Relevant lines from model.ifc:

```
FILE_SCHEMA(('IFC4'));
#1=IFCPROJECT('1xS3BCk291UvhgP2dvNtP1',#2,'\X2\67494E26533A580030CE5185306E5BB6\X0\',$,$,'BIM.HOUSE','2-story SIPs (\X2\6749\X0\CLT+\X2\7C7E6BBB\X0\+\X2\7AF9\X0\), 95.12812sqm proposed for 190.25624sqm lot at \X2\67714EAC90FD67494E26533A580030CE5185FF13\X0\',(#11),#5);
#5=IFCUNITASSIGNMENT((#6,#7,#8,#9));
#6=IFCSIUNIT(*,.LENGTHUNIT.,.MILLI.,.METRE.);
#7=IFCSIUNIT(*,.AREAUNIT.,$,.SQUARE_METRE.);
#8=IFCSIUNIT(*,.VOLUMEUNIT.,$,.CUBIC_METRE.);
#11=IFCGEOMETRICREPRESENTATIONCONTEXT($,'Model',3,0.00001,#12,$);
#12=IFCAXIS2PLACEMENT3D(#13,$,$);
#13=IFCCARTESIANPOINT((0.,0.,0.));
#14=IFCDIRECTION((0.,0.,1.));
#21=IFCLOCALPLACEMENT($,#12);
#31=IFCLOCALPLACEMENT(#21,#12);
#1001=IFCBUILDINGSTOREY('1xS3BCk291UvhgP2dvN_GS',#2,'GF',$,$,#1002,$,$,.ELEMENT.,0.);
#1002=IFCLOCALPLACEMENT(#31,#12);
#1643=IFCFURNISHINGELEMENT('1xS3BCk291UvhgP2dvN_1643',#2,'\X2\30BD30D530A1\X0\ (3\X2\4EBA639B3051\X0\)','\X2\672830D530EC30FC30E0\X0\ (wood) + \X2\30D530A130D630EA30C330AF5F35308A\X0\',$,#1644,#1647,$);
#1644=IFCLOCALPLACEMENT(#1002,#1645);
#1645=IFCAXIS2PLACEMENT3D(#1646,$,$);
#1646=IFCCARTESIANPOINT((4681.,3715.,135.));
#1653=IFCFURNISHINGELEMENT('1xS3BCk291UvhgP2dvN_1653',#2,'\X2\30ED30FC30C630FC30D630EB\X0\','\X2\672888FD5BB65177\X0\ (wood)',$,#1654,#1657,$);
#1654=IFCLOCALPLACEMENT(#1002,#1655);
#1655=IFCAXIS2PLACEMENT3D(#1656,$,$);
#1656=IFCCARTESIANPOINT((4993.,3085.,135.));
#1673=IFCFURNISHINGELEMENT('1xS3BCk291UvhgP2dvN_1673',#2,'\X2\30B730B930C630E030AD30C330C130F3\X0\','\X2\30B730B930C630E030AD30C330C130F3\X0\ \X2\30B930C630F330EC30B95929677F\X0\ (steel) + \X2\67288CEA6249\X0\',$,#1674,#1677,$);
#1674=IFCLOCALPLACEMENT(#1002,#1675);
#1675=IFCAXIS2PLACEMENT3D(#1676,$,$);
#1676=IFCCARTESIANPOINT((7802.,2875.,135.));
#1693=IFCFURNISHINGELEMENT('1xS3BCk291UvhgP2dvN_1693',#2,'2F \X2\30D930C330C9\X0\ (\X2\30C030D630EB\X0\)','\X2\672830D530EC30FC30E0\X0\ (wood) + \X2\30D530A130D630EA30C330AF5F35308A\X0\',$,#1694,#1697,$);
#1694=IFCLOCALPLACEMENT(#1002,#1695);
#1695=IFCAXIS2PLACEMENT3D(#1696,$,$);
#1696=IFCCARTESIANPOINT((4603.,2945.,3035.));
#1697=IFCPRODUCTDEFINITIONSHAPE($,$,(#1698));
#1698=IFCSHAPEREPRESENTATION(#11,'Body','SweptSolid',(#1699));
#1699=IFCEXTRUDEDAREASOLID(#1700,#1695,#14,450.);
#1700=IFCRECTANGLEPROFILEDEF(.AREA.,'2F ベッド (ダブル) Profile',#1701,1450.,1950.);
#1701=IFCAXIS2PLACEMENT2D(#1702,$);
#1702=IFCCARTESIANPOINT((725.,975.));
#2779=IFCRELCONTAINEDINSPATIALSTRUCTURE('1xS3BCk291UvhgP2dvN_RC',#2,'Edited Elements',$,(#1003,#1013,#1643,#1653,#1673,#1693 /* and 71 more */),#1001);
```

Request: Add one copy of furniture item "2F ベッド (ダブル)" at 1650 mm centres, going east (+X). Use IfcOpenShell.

```python
import numpy as np
import ifcopenshell
import ifcopenshell.api.geometry
import ifcopenshell.api.root
import ifcopenshell.util.element
import ifcopenshell.util.placement
import ifcopenshell.util.unit

model = ifcopenshell.open("model.ifc")
unit_scale = ifcopenshell.util.unit.calculate_unit_scale(model)


def reuse_history(source, copy):
    """copy_class also copies each property set's owner history, people and application; keep the originals."""
    for rel in copy.IsDefinedBy:
        if rel.is_a("IfcRelDefinesByProperties") and (history := rel.RelatingPropertyDefinition.OwnerHistory):
            rel.RelatingPropertyDefinition.OwnerHistory = source.OwnerHistory
            ifcopenshell.util.element.remove_deep2(model, history)


source = model.by_guid("1xS3BCk291UvhgP2dvN_1693")
base = ifcopenshell.util.placement.get_local_placement(source.ObjectPlacement)
step = np.array([1.0, 0.0, 0.0]) * 1.65 / unit_scale

for i in range(1, 2):
    copy = ifcopenshell.api.root.copy_class(model, product=source)
    copy.Representation = ifcopenshell.util.element.copy_deep(
        model, source.Representation, exclude=["IfcGeometricRepresentationContext", "IfcRepresentationMap"]
    )
    reuse_history(source, copy)
    matrix = base.copy()
    matrix[:3, 3] += i * step
    print("added at", matrix[:3, 3].round(3) + 0.0)
    ifcopenshell.api.geometry.edit_object_placement(model, product=copy, matrix=matrix, is_si=False)

model.write("model_rev.ifc")
```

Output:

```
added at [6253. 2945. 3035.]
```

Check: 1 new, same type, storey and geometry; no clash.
